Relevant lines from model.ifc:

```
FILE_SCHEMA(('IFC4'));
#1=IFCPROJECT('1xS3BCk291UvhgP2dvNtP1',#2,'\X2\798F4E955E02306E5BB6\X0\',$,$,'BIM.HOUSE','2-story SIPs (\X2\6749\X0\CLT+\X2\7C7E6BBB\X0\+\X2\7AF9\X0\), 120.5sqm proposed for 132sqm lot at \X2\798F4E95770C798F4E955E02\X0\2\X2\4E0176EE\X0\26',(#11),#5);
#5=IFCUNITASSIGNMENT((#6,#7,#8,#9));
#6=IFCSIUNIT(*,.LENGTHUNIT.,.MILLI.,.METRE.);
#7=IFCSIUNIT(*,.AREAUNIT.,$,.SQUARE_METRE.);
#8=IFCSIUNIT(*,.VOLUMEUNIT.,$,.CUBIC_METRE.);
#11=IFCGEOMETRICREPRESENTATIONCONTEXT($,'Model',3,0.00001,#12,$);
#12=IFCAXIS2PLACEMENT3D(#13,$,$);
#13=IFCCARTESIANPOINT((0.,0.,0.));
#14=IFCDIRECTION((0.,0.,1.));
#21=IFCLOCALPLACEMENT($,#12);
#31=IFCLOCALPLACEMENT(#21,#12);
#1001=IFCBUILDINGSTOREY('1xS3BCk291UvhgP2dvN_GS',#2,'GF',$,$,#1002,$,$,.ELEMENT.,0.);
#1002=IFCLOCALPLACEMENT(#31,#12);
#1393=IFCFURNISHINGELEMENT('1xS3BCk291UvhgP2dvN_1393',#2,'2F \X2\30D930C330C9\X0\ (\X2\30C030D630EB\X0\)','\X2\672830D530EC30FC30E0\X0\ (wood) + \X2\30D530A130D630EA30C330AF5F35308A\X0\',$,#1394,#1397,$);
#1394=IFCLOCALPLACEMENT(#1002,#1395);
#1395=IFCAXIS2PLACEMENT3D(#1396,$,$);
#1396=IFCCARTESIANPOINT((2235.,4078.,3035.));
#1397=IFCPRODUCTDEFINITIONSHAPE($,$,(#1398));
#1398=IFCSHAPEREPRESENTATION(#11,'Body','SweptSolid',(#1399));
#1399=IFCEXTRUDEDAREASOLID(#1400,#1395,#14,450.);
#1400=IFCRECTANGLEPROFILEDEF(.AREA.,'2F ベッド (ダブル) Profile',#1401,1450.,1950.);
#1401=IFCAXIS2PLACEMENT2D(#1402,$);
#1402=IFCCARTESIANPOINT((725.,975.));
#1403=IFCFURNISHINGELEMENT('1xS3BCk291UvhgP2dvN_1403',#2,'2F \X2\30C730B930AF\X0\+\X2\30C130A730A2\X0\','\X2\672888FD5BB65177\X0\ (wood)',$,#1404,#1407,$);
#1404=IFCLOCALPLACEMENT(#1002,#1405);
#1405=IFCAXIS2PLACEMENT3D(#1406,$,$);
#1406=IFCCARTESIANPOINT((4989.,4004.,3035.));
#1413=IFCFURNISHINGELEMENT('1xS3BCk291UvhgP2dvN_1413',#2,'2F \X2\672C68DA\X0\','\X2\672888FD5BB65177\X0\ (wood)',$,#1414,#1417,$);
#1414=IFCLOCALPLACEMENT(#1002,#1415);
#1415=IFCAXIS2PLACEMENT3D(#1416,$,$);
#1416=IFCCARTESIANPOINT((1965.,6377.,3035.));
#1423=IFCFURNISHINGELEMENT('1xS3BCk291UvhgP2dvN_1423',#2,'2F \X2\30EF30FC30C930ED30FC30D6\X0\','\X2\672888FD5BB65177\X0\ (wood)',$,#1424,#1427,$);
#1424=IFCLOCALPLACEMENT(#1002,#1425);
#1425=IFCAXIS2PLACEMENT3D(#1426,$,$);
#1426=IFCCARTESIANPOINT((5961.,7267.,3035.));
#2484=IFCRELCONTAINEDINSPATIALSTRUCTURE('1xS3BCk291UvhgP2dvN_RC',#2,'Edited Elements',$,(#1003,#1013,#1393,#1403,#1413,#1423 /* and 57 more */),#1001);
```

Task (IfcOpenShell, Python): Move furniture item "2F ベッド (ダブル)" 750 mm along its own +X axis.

```python
import ifcopenshell
import ifcopenshell.api.geometry
import ifcopenshell.util.placement
import ifcopenshell.util.unit

model = ifcopenshell.open("model.ifc")
unit_scale = ifcopenshell.util.unit.calculate_unit_scale(model)

item = model.by_guid("1xS3BCk291UvhgP2dvN_1393")
matrix = ifcopenshell.util.placement.get_local_placement(item.ObjectPlacement)
matrix[:3, 3] += matrix[:3, 0] * 0.75 / unit_scale
ifcopenshell.api.geometry.edit_object_placement(model, product=item, matrix=matrix, is_si=False)

print(ifcopenshell.util.placement.get_local_placement(item.ObjectPlacement).round(3) + 0.0)

model.write("model_edited.ifc")
```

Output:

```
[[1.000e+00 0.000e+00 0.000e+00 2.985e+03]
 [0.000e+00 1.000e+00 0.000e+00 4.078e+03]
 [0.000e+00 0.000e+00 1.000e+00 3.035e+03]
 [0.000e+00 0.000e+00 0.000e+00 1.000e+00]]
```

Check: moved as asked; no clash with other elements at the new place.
